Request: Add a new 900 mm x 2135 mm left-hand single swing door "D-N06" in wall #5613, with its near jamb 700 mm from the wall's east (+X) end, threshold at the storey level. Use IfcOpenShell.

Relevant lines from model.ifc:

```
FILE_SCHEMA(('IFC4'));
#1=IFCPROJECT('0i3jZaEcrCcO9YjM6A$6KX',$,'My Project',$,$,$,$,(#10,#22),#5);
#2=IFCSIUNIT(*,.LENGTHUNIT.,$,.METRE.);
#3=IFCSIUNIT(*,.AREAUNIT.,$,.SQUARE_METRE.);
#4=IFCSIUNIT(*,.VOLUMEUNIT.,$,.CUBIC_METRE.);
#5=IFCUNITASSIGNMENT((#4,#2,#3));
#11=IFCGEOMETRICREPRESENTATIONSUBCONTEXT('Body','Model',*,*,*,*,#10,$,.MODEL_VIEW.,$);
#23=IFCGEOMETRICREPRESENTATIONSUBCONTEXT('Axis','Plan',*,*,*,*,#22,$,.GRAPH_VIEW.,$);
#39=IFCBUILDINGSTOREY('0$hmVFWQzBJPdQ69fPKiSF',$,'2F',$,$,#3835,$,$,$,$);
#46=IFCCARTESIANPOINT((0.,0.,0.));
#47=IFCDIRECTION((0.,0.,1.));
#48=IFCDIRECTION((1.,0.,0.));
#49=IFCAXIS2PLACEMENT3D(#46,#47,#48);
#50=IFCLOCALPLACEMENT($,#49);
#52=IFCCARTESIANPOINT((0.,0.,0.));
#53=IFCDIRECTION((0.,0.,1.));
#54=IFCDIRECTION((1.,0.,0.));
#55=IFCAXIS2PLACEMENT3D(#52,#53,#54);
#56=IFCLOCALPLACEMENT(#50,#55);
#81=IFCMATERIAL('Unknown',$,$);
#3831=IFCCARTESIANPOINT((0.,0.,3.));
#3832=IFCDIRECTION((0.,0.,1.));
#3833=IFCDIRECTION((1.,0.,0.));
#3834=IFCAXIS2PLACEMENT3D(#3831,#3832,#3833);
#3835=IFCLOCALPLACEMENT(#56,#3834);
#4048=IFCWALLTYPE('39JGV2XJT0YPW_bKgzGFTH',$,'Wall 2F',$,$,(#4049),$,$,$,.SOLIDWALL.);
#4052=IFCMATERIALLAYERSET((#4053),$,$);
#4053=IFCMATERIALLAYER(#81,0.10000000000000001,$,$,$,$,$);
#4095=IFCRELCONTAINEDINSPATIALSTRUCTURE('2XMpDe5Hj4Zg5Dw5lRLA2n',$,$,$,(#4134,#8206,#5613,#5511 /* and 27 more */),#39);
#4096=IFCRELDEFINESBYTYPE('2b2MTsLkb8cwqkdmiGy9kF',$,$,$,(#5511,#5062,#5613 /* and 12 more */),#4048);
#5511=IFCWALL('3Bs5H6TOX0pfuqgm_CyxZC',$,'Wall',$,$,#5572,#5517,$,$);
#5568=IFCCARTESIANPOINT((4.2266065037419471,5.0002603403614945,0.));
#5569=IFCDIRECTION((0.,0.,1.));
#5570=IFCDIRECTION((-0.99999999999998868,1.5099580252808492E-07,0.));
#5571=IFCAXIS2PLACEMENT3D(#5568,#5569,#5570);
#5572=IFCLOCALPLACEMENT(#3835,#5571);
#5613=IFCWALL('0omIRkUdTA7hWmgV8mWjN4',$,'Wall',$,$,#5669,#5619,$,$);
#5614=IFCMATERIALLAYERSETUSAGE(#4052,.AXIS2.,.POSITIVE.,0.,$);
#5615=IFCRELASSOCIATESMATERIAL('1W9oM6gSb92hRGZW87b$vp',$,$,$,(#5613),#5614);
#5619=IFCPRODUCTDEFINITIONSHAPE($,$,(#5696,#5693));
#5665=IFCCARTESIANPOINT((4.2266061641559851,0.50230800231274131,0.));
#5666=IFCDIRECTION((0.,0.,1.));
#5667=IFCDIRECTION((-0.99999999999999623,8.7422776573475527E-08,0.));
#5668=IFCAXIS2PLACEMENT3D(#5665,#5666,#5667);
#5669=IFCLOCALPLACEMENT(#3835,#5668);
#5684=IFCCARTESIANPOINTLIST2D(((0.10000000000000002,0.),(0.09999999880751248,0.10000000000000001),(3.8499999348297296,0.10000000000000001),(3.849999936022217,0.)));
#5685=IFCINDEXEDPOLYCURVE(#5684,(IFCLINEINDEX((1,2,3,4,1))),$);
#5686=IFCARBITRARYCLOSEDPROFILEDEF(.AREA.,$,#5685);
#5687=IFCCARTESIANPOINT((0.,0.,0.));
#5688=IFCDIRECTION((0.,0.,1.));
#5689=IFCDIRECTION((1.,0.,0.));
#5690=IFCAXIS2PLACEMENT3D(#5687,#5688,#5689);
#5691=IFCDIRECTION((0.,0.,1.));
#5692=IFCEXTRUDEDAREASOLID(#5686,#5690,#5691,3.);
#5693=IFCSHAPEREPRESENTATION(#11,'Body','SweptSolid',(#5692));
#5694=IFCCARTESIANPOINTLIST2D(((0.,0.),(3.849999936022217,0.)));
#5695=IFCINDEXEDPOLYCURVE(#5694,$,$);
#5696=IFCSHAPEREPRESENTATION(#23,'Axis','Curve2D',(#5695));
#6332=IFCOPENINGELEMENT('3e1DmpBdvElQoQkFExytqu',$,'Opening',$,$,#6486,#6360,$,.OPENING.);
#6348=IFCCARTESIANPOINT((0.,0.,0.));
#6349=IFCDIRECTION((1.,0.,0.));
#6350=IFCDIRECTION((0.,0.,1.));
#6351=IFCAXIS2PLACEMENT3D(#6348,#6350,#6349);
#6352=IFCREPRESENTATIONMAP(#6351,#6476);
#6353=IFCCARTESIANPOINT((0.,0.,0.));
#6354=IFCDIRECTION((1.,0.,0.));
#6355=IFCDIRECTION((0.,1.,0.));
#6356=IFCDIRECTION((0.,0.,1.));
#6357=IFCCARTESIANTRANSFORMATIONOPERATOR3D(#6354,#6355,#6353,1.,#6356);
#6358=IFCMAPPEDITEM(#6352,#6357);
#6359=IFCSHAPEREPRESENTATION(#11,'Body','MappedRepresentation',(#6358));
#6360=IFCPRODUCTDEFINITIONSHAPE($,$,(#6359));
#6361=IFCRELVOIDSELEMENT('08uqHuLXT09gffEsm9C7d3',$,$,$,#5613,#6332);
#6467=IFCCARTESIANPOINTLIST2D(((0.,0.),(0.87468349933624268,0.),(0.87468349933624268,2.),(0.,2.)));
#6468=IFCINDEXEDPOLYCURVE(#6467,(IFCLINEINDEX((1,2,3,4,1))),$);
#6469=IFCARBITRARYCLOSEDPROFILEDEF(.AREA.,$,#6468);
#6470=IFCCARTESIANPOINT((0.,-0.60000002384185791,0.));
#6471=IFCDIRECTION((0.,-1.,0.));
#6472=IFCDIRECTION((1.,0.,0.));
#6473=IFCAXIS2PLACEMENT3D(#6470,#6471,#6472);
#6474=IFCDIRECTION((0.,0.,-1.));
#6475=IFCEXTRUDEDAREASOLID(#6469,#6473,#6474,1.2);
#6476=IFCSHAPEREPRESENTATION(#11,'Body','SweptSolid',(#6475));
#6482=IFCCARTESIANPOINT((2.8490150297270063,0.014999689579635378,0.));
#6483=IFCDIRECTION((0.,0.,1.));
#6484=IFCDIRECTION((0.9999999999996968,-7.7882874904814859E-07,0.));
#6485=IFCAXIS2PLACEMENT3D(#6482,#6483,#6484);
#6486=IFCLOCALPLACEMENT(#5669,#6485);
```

```python
import numpy as np
import ifcopenshell
import ifcopenshell.api.feature
import ifcopenshell.api.geometry
import ifcopenshell.api.root
import ifcopenshell.api.spatial
import ifcopenshell.geom
import ifcopenshell.util.element
import ifcopenshell.util.placement
import ifcopenshell.util.representation
import ifcopenshell.util.shape
import ifcopenshell.util.unit

model = ifcopenshell.open("model.ifc")
unit_scale = ifcopenshell.util.unit.calculate_unit_scale(model)
settings = ifcopenshell.geom.settings()


def volume(element):
    """Net volume in cubic metres, openings subtracted."""
    shape = ifcopenshell.geom.create_shape(settings, element)
    return ifcopenshell.util.shape.get_volume(shape.geometry)


wall = model.by_guid("0omIRkUdTA7hWmgV8mWjN4")
storey = ifcopenshell.util.element.get_container(wall, ifc_class="IfcBuildingStorey")
context = ifcopenshell.util.representation.get_context(model, "Model", "Body", "MODEL_VIEW")
before = volume(wall)

width, height, from_end, sill = 0.9, 2.135, 0.7, 0.0  # metres

# The wall runs along its own X axis, and the end named is its -X end.
wall_shape = ifcopenshell.geom.create_shape(settings, wall)
x, y, z = ifcopenshell.util.shape.get_vertices(wall_shape.geometry).T
start = x.min() + from_end
face, thickness = float(y.min()), float(y.max() - y.min())
wall_matrix = ifcopenshell.util.placement.get_local_placement(wall.ObjectPlacement)
level = ifcopenshell.util.placement.get_local_placement(storey.ObjectPlacement)[2, 3]


def in_wall(x, y):
    """Placement at x, y metres in the wall's axes, at sill height."""
    matrix = wall_matrix.copy()
    matrix[:, 3] = wall_matrix @ np.array([x / unit_scale, y / unit_scale, 0.0, 1.0])
    matrix[2, 3] = level + sill / unit_scale
    return matrix


# Opening: a box that overshoots both wall faces by 50 mm.
opening = ifcopenshell.api.root.create_entity(model, ifc_class="IfcOpeningElement", predefined_type="OPENING")
box = ifcopenshell.api.geometry.add_wall_representation(
    model, context=context, length=width, height=height, thickness=thickness + 0.1
)
ifcopenshell.api.geometry.assign_representation(model, product=opening, representation=box)
ifcopenshell.api.geometry.edit_object_placement(model, product=opening, matrix=in_wall(start, face - 0.05), is_si=False)
ifcopenshell.api.feature.add_feature(model, feature=opening, element=wall)

door = ifcopenshell.api.root.create_entity(model, ifc_class="IfcDoor", name="D-N06", predefined_type="DOOR")
door.OverallWidth, door.OverallHeight = width / unit_scale, height / unit_scale
door.OperationType = "SINGLE_SWING_LEFT"
body = ifcopenshell.api.geometry.add_door_representation(
    model,
    context=context,
    overall_width=door.OverallWidth,
    overall_height=door.OverallHeight,
    operation_type="SINGLE_SWING_LEFT",
    lining_properties={"LiningDepth": thickness / unit_scale, "ThresholdDepth": thickness / unit_scale},
)
ifcopenshell.api.geometry.assign_representation(model, product=door, representation=body)
ifcopenshell.api.spatial.assign_container(model, products=[door], relating_structure=storey)
ifcopenshell.api.feature.add_filling(model, opening=opening, element=door)

# The lining spans the wall, so the door starts at the wall face.
ifcopenshell.api.geometry.edit_object_placement(model, product=door, matrix=in_wall(start, face), is_si=False)

after = volume(wall)

print(f"wall volume {before:.3f} -> {after:.3f} m3")

model.write("model_updated.ifc")
```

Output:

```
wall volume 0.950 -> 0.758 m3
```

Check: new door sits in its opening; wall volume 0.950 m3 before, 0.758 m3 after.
